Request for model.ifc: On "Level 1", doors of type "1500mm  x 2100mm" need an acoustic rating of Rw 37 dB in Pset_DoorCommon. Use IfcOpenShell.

First a look at what the model holds.

```python
import ifcopenshell
import ifcopenshell.util.element

model = ifcopenshell.open("model.ifc")
print(model.schema)
storey = next(s for s in model.by_type("IfcBuildingStorey") if s.Name == "Level 1")
doors = [e for e in ifcopenshell.util.element.get_decomposition(storey) if e.is_a("IfcDoor")]
seen = {}
for e in doors:
    element_type = ifcopenshell.util.element.get_type(e)
    key = (element_type.Name if element_type != e and element_type else None, ifcopenshell.util.element.get_pset(e, "Pset_DoorCommon", "AcousticRating"))
    seen[key] = seen.get(key, 0) + 1
for (name, value), count in sorted(seen.items(), key=str):
    print(count, "x", name, "|", value)
```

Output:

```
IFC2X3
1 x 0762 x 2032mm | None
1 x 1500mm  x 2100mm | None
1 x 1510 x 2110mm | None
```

```python
import ifcopenshell
import ifcopenshell.api.pset
import ifcopenshell.util.element

model = ifcopenshell.open("model.ifc")

storey = next(s for s in model.by_type("IfcBuildingStorey") if s.Name == "Level 1")
doors = [e for e in ifcopenshell.util.element.get_decomposition(storey) if e.is_a("IfcDoor")]

count = 0
for e in doors:
    element_type = ifcopenshell.util.element.get_type(e)
    if element_type in (None, e) or element_type.Name != "1500mm  x 2100mm":
        continue
    # add_pset returns the element's existing set when there is one.
    pset = ifcopenshell.api.pset.add_pset(model, product=e, name="Pset_DoorCommon")
    ifcopenshell.api.pset.edit_pset(model, pset=pset, properties={"AcousticRating": "Rw 37 dB"})
    count += 1

print(count, "doors updated")

model.write("model-out.ifc")
```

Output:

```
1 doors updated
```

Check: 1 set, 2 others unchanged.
